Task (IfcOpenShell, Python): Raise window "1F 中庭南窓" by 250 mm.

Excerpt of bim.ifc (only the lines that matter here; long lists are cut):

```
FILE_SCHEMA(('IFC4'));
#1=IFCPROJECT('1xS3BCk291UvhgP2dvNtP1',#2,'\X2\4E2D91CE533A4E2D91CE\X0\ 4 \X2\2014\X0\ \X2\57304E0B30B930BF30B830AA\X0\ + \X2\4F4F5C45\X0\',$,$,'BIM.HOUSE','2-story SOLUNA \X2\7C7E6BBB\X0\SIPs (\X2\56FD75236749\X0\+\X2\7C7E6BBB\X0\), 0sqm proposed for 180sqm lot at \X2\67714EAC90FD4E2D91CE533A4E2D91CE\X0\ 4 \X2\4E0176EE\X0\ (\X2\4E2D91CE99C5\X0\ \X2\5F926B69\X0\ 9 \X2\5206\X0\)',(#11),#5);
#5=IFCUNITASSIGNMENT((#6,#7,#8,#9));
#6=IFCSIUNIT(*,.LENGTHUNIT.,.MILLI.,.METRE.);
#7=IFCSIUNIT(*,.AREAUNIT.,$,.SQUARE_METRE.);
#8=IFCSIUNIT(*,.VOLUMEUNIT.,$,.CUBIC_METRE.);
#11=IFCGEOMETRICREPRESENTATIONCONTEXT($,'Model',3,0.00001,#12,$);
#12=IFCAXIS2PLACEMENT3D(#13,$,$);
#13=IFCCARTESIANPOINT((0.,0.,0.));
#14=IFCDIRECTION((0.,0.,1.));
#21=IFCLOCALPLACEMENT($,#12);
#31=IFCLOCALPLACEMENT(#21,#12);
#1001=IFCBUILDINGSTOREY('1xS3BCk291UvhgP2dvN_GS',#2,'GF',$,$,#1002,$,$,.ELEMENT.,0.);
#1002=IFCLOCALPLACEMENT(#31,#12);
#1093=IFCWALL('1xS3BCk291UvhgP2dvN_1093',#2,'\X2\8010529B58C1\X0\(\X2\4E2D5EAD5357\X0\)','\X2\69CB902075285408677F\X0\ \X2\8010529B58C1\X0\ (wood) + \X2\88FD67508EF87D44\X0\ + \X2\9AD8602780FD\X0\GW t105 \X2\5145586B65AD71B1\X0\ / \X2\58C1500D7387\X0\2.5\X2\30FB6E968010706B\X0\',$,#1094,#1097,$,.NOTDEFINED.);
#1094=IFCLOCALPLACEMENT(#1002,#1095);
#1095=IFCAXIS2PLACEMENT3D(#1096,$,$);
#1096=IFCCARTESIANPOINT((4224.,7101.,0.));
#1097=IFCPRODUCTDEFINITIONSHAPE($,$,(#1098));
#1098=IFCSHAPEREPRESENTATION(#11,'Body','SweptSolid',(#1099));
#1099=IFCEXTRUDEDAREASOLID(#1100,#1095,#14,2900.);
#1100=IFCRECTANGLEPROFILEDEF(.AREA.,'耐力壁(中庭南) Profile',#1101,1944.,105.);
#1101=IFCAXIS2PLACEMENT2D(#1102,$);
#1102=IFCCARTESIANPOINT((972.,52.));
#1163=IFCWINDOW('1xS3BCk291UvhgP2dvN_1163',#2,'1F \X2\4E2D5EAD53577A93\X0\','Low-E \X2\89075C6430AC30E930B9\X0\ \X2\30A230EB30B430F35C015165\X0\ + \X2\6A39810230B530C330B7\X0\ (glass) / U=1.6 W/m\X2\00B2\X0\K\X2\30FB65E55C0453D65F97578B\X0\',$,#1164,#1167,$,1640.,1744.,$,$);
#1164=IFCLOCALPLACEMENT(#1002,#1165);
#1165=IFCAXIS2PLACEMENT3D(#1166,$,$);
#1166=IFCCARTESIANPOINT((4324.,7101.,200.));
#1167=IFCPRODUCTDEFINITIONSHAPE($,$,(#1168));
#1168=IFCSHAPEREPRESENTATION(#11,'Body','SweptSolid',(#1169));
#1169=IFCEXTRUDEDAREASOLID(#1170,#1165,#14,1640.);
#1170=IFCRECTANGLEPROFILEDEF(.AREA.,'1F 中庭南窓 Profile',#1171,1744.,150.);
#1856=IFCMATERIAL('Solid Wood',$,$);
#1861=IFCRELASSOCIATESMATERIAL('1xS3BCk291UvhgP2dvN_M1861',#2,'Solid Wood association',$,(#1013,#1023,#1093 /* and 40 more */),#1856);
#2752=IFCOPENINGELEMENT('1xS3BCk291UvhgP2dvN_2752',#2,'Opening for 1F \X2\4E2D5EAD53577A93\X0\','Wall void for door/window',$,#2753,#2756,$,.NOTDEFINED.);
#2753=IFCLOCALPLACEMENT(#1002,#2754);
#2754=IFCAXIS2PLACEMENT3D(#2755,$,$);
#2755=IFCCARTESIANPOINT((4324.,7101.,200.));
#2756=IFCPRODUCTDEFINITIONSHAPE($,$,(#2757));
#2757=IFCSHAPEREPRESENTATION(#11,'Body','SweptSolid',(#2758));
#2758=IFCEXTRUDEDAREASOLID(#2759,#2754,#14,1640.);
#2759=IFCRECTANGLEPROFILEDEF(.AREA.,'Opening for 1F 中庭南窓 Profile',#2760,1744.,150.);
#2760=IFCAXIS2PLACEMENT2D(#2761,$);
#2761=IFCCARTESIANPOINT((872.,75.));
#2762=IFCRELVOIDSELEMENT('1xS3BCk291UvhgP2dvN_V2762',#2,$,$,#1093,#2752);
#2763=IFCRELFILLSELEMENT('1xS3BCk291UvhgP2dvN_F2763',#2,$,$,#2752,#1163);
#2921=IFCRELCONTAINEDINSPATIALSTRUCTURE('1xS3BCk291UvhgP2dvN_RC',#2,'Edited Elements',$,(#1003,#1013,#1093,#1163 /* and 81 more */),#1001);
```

```python
import numpy as np
import ifcopenshell
import ifcopenshell.api.geometry
import ifcopenshell.util.placement
import ifcopenshell.util.unit

model = ifcopenshell.open("bim.ifc")
unit_scale = ifcopenshell.util.unit.calculate_unit_scale(model)

window = model.by_guid("1xS3BCk291UvhgP2dvN_1163")
opening = window.FillsVoids[0].RelatingOpeningElement
dz = 0.25 / unit_scale

shift = np.array([0.0, 0.0, dz])
# The window is not placed relative to its opening, so move both.
for product in (opening, window):
    matrix = ifcopenshell.util.placement.get_local_placement(product.ObjectPlacement)
    matrix[:3, 3] += shift
    ifcopenshell.api.geometry.edit_object_placement(model, product=product, matrix=matrix, is_si=False)

print(f"moved by {dz * unit_scale:+.3f} m")

model.write("bim_rev.ifc")
```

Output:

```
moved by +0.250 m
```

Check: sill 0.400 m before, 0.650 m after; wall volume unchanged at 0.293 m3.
